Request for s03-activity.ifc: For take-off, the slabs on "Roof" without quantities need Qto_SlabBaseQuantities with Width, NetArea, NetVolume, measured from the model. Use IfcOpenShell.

First a look at what the model holds.

```python
import ifcopenshell
import ifcopenshell.util.element
import ifcopenshell.util.unit

model = ifcopenshell.open("s03-activity.ifc")
print(model.schema)
for unit_type in ("LENGTHUNIT", "AREAUNIT", "VOLUMEUNIT"):
    print(unit_type, ifcopenshell.util.unit.calculate_unit_scale(model, unit_type))
storey = next(s for s in model.by_type("IfcBuildingStorey") if s.Name == "Roof")
slabs = [e for e in ifcopenshell.util.element.get_decomposition(storey) if e.is_a("IfcSlab")]
for e in sorted(slabs, key=lambda e: e.id()):
    print(e.id(), e.is_a(), e.Name, list(ifcopenshell.util.element.get_psets(e, qtos_only=True)), sep=" | ")
```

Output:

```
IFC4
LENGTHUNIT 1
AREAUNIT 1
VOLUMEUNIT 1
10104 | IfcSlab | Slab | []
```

```python
import ifcopenshell
import ifcopenshell.api.pset
import ifcopenshell.geom
import ifcopenshell.util.element
import ifcopenshell.util.shape
import ifcopenshell.util.unit

model = ifcopenshell.open("s03-activity.ifc")
unit_scale = ifcopenshell.util.unit.calculate_unit_scale(model)
area_scale = ifcopenshell.util.unit.calculate_unit_scale(model, "AREAUNIT")
volume_scale = ifcopenshell.util.unit.calculate_unit_scale(model, "VOLUMEUNIT")
settings = ifcopenshell.geom.settings()

storey = next(s for s in model.by_type("IfcBuildingStorey") if s.Name == "Roof")
slabs = [e for e in ifcopenshell.util.element.get_decomposition(storey) if e.is_a("IfcSlab")]

for e in sorted(slabs, key=lambda e: e.id()):
    if ifcopenshell.util.element.get_psets(e, qtos_only=True, should_inherit=False):
        continue
    # Geometry comes back in metres, in the element's own axes.
    shape = ifcopenshell.geom.create_shape(settings, e)
    values = {
        "Width": ifcopenshell.util.shape.get_z(shape.geometry) / unit_scale,
        "NetArea": ifcopenshell.util.shape.get_footprint_area(shape.geometry) / area_scale,
        "NetVolume": ifcopenshell.util.shape.get_volume(shape.geometry) / volume_scale,
    }
    qto = ifcopenshell.api.pset.add_qto(model, product=e, name="Qto_SlabBaseQuantities")
    ifcopenshell.api.pset.edit_qto(model, qto=qto, properties=values)
    print(e.id(), {k: round(v, 3) for k, v in values.items()})

model.write("s03-activity_updated.ifc")
```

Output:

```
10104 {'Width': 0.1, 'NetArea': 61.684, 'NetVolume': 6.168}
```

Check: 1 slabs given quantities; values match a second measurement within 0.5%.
